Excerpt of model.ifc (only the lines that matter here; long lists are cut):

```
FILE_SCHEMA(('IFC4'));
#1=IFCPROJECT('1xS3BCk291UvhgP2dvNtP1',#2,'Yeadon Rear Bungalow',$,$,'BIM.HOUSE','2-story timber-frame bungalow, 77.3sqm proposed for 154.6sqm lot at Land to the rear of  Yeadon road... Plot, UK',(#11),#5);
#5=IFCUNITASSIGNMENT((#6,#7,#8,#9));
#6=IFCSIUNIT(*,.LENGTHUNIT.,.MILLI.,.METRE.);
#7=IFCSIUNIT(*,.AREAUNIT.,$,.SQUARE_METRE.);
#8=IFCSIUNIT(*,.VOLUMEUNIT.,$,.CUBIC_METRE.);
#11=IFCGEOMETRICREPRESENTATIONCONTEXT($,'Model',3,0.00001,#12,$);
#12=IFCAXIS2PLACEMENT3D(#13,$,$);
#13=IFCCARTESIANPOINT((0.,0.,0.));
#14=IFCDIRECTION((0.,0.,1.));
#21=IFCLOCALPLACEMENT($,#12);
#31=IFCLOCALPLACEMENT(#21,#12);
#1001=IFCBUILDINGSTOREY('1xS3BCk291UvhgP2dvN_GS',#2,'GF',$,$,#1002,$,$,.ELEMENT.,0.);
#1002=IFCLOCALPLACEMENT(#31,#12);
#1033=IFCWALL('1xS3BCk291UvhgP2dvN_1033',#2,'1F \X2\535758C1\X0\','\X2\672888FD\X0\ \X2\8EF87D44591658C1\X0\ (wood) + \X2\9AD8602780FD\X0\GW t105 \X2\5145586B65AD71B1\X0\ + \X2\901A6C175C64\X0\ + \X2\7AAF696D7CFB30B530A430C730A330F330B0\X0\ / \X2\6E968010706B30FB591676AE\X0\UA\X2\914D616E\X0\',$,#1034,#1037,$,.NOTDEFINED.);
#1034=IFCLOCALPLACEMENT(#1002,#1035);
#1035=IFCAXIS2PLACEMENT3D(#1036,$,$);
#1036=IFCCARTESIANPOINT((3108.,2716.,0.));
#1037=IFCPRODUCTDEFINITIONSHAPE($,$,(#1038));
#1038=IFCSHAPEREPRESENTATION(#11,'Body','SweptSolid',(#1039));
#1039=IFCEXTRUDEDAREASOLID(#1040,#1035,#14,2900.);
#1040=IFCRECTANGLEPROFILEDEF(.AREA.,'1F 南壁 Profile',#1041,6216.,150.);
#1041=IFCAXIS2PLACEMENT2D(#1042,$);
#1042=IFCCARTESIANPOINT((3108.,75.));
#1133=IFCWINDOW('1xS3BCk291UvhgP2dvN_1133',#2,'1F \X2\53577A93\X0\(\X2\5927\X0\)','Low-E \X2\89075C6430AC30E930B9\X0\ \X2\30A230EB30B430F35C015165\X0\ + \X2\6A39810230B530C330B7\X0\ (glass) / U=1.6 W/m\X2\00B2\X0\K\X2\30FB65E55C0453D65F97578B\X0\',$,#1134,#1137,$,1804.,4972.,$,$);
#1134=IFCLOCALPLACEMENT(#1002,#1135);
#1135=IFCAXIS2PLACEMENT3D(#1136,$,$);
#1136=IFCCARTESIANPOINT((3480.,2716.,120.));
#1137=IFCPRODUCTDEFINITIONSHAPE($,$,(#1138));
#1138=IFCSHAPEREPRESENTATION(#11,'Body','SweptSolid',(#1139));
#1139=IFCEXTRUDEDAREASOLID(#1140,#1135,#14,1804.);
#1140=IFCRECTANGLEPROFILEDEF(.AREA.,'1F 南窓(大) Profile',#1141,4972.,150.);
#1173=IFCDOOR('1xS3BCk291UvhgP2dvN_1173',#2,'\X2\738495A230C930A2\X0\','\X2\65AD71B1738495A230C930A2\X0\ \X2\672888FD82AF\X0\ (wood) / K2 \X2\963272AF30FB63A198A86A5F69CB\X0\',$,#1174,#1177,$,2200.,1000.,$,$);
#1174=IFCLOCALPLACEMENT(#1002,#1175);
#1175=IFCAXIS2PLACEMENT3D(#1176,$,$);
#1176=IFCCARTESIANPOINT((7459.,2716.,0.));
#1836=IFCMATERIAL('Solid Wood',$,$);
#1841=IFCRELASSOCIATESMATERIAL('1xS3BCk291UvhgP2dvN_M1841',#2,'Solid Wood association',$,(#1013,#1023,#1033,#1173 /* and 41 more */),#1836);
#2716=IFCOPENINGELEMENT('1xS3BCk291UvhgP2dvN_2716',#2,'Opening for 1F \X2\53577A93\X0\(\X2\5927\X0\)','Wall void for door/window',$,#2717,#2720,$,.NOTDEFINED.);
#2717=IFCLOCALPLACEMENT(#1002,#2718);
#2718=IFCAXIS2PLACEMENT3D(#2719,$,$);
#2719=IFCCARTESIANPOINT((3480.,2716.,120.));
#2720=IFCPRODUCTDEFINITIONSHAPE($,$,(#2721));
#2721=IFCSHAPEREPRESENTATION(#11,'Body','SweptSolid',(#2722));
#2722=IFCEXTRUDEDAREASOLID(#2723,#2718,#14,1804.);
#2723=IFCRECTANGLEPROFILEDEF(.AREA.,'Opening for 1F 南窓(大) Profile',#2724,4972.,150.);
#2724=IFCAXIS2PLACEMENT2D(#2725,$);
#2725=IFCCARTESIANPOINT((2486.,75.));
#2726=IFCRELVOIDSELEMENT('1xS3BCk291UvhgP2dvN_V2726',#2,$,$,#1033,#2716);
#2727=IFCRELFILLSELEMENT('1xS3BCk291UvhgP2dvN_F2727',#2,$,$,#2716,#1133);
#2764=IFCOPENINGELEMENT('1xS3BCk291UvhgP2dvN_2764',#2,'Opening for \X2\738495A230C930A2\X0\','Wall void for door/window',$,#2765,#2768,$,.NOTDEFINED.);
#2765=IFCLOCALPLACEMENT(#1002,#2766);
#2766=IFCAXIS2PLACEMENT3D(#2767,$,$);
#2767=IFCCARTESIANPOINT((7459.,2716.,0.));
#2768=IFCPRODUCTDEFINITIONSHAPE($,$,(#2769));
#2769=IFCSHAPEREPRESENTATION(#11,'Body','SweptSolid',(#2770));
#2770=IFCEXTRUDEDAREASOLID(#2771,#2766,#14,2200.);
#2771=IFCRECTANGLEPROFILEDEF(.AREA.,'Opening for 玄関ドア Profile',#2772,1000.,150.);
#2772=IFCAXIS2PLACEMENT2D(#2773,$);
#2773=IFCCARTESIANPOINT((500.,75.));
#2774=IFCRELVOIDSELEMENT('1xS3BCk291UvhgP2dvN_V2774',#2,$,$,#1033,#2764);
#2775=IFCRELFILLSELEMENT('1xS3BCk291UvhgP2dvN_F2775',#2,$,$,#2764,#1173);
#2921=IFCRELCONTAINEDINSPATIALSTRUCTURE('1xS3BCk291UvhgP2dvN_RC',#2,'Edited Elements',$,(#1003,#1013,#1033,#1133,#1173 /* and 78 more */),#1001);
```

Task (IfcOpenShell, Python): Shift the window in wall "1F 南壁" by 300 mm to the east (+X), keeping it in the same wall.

```python
import ifcopenshell
import ifcopenshell.api.geometry
import ifcopenshell.util.placement
import ifcopenshell.util.unit

model = ifcopenshell.open("model.ifc")
unit_scale = ifcopenshell.util.unit.calculate_unit_scale(model)

window = model.by_guid("1xS3BCk291UvhgP2dvN_1133")
opening = window.FillsVoids[0].RelatingOpeningElement
wall = opening.VoidsElements[0].RelatingBuildingElement

wall_matrix = ifcopenshell.util.placement.get_local_placement(wall.ObjectPlacement)
shift = wall_matrix[:3, 0] * 0.3 / unit_scale
before = ifcopenshell.util.placement.get_local_placement(window.ObjectPlacement)[:3, 3].copy()

# The window is not placed relative to its opening, so move both.
for product in (opening, window):
    matrix = ifcopenshell.util.placement.get_local_placement(product.ObjectPlacement)
    matrix[:3, 3] += shift
    ifcopenshell.api.geometry.edit_object_placement(model, product=product, matrix=matrix, is_si=False)

after = ifcopenshell.util.placement.get_local_placement(window.ObjectPlacement)[:3, 3]
print("window moved by", (after - before).round(3) + 0.0)

model.write("model_v2.ifc")
```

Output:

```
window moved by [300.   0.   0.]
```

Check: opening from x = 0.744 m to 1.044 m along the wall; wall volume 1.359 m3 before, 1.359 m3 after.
